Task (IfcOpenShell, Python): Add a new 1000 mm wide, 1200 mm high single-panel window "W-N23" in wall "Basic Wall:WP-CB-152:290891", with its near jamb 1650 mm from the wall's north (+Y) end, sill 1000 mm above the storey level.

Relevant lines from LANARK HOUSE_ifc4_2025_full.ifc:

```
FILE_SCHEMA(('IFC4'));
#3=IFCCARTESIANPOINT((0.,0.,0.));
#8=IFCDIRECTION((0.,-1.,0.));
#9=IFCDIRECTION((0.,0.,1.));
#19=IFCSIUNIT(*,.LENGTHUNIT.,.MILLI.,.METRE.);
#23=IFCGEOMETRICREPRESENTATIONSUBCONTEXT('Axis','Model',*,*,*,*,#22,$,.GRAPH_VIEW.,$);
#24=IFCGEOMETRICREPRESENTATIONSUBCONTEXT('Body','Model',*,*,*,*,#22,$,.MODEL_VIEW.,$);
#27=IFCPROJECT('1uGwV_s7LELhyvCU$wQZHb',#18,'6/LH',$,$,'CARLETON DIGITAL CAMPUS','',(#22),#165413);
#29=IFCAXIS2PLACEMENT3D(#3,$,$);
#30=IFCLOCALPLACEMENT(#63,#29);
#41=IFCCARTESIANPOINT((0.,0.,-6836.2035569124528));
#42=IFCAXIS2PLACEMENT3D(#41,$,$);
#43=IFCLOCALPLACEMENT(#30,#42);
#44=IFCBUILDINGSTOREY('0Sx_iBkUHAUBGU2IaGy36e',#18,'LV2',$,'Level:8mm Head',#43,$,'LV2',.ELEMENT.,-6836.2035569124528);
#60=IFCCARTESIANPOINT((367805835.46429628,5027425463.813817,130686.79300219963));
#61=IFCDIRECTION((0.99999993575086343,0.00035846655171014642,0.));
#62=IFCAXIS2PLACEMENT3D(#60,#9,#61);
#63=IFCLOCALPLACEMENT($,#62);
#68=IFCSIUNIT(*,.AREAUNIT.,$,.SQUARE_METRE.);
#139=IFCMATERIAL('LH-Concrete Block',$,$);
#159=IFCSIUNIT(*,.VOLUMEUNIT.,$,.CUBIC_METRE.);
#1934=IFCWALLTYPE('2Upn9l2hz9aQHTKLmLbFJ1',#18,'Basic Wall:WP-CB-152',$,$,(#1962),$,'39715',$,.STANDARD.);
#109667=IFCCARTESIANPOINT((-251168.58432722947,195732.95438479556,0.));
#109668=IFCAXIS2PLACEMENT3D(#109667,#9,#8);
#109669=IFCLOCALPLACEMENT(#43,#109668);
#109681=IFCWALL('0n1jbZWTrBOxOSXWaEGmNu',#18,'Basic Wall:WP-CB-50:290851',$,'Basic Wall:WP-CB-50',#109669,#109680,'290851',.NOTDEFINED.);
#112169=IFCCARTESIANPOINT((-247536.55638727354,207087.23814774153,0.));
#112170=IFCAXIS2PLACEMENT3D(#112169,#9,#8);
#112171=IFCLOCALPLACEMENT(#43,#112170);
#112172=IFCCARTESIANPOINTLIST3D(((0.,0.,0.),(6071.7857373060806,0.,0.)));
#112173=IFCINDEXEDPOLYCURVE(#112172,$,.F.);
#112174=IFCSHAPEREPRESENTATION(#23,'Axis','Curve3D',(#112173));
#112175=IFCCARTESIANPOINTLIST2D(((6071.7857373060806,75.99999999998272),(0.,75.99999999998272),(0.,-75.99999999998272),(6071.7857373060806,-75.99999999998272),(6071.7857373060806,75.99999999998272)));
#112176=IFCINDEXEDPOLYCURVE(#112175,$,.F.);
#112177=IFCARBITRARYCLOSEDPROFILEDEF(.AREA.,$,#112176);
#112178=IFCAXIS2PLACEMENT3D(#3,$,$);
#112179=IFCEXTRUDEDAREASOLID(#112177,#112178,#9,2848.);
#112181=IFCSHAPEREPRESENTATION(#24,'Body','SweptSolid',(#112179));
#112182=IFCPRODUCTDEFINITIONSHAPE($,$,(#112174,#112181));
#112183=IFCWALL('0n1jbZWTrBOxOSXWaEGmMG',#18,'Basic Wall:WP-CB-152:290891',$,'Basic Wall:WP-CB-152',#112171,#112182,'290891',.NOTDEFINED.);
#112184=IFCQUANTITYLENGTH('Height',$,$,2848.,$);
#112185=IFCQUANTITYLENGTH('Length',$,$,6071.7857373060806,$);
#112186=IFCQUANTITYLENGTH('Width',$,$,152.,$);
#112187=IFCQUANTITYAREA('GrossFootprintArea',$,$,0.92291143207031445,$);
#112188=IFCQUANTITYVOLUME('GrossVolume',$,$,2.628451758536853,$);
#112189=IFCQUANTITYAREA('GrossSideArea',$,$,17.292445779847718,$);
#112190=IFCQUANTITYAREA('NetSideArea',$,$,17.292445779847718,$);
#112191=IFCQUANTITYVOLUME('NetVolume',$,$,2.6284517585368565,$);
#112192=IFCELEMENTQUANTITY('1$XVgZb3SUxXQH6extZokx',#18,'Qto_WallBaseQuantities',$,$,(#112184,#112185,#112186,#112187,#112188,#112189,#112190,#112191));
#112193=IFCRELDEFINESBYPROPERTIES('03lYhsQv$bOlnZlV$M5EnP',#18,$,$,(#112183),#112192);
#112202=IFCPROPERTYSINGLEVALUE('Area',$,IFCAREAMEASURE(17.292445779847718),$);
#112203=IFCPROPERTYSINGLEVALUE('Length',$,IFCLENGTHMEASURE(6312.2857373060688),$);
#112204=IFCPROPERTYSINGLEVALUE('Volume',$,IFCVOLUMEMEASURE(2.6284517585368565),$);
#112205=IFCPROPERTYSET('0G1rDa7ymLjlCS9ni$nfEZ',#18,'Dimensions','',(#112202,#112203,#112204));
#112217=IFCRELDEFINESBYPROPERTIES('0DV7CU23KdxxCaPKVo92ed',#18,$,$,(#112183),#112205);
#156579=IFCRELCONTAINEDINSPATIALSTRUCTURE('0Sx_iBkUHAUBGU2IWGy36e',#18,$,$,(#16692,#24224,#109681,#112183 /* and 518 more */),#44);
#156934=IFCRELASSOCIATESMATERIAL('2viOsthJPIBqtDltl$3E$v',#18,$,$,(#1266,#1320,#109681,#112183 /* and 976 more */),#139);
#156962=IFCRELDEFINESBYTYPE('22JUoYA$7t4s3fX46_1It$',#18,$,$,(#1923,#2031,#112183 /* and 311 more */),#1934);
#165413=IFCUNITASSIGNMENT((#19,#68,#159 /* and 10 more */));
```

```python
import numpy as np
import ifcopenshell
import ifcopenshell.api.feature
import ifcopenshell.api.geometry
import ifcopenshell.api.pset
import ifcopenshell.api.root
import ifcopenshell.api.spatial
import ifcopenshell.geom
import ifcopenshell.util.element
import ifcopenshell.util.placement
import ifcopenshell.util.representation
import ifcopenshell.util.shape
import ifcopenshell.util.unit

model = ifcopenshell.open("LANARK HOUSE_ifc4_2025_full.ifc")
unit_scale = ifcopenshell.util.unit.calculate_unit_scale(model)
area_scale = ifcopenshell.util.unit.calculate_unit_scale(model, "AREAUNIT")
volume_scale = ifcopenshell.util.unit.calculate_unit_scale(model, "VOLUMEUNIT")
settings = ifcopenshell.geom.settings()


def volume(element):
    """Net volume in cubic metres, openings subtracted."""
    shape = ifcopenshell.geom.create_shape(settings, element)
    return ifcopenshell.util.shape.get_volume(shape.geometry)


wall = model.by_guid("0n1jbZWTrBOxOSXWaEGmMG")
storey = ifcopenshell.util.element.get_container(wall, ifc_class="IfcBuildingStorey")
context = ifcopenshell.util.representation.get_context(model, "Model", "Body", "MODEL_VIEW")
before = volume(wall)

width, height, from_end, sill = 1, 1.2, 1.65, 1  # metres

# The wall runs along its own X axis, and the end named is its -X end.
wall_shape = ifcopenshell.geom.create_shape(settings, wall)
x, y, z = ifcopenshell.util.shape.get_vertices(wall_shape.geometry).T
start = x.min() + from_end
face, thickness = float(y.min()), float(y.max() - y.min())
wall_matrix = ifcopenshell.util.placement.get_local_placement(wall.ObjectPlacement)
level = ifcopenshell.util.placement.get_local_placement(storey.ObjectPlacement)[2, 3]


def in_wall(x, y):
    """Placement at x, y metres in the wall's axes, at sill height."""
    matrix = wall_matrix.copy()
    matrix[:, 3] = wall_matrix @ np.array([x / unit_scale, y / unit_scale, 0.0, 1.0])
    matrix[2, 3] = level + sill / unit_scale
    return matrix


# Opening: a box that overshoots both wall faces by 50 mm.
opening = ifcopenshell.api.root.create_entity(model, ifc_class="IfcOpeningElement", predefined_type="OPENING")
box = ifcopenshell.api.geometry.add_wall_representation(
    model, context=context, length=width, height=height, thickness=thickness + 0.1
)
ifcopenshell.api.geometry.assign_representation(model, product=opening, representation=box)
ifcopenshell.api.geometry.edit_object_placement(model, product=opening, matrix=in_wall(start, face - 0.05), is_si=False)
ifcopenshell.api.feature.add_feature(model, feature=opening, element=wall)

window = ifcopenshell.api.root.create_entity(model, ifc_class="IfcWindow", name="W-N23", predefined_type="WINDOW")
window.OverallWidth, window.OverallHeight = width / unit_scale, height / unit_scale
window.PartitioningType = "SINGLE_PANEL"
body = ifcopenshell.api.geometry.add_window_representation(
    model,
    context=context,
    overall_width=window.OverallWidth,
    overall_height=window.OverallHeight,
    partition_type="SINGLE_PANEL",
)
ifcopenshell.api.geometry.assign_representation(model, product=window, representation=body)
ifcopenshell.api.spatial.assign_container(model, products=[window], relating_structure=storey)
ifcopenshell.api.feature.add_filling(model, opening=opening, element=window)

# Centre the window in the wall's thickness.
ifcopenshell.api.geometry.edit_object_placement(model, product=window, matrix=in_wall(start, face), is_si=False)
window_shape = ifcopenshell.geom.create_shape(settings, window)
depth = ifcopenshell.util.shape.get_vertices(window_shape.geometry)[:, 1]
offset = face + thickness / 2 - (depth.min() + depth.max()) / 2
ifcopenshell.api.geometry.edit_object_placement(model, product=window, matrix=in_wall(start, offset), is_si=False)

after = volume(wall)

# Update the wall's stored quantities.
qto = model.by_id(ifcopenshell.util.element.get_pset(wall, "Qto_WallBaseQuantities", should_inherit=False)["id"])
ifcopenshell.api.pset.edit_qto(model, qto=qto, properties={
    "NetSideArea": after / thickness / area_scale,
    "NetVolume": after / volume_scale,
})
pset = model.by_id(ifcopenshell.util.element.get_pset(wall, "Dimensions", should_inherit=False)["id"])
ifcopenshell.api.pset.edit_pset(model, pset=pset, properties={
    "Area": model.create_entity("IfcAreaMeasure", after / thickness / area_scale),
    "Volume": model.create_entity("IfcVolumeMeasure", after / volume_scale),
})

print(f"wall volume {before:.3f} -> {after:.3f} m3")

model.write("LANARK HOUSE_ifc4_2025_full_edited.ifc")
```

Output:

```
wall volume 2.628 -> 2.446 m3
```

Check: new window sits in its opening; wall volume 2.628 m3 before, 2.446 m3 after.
